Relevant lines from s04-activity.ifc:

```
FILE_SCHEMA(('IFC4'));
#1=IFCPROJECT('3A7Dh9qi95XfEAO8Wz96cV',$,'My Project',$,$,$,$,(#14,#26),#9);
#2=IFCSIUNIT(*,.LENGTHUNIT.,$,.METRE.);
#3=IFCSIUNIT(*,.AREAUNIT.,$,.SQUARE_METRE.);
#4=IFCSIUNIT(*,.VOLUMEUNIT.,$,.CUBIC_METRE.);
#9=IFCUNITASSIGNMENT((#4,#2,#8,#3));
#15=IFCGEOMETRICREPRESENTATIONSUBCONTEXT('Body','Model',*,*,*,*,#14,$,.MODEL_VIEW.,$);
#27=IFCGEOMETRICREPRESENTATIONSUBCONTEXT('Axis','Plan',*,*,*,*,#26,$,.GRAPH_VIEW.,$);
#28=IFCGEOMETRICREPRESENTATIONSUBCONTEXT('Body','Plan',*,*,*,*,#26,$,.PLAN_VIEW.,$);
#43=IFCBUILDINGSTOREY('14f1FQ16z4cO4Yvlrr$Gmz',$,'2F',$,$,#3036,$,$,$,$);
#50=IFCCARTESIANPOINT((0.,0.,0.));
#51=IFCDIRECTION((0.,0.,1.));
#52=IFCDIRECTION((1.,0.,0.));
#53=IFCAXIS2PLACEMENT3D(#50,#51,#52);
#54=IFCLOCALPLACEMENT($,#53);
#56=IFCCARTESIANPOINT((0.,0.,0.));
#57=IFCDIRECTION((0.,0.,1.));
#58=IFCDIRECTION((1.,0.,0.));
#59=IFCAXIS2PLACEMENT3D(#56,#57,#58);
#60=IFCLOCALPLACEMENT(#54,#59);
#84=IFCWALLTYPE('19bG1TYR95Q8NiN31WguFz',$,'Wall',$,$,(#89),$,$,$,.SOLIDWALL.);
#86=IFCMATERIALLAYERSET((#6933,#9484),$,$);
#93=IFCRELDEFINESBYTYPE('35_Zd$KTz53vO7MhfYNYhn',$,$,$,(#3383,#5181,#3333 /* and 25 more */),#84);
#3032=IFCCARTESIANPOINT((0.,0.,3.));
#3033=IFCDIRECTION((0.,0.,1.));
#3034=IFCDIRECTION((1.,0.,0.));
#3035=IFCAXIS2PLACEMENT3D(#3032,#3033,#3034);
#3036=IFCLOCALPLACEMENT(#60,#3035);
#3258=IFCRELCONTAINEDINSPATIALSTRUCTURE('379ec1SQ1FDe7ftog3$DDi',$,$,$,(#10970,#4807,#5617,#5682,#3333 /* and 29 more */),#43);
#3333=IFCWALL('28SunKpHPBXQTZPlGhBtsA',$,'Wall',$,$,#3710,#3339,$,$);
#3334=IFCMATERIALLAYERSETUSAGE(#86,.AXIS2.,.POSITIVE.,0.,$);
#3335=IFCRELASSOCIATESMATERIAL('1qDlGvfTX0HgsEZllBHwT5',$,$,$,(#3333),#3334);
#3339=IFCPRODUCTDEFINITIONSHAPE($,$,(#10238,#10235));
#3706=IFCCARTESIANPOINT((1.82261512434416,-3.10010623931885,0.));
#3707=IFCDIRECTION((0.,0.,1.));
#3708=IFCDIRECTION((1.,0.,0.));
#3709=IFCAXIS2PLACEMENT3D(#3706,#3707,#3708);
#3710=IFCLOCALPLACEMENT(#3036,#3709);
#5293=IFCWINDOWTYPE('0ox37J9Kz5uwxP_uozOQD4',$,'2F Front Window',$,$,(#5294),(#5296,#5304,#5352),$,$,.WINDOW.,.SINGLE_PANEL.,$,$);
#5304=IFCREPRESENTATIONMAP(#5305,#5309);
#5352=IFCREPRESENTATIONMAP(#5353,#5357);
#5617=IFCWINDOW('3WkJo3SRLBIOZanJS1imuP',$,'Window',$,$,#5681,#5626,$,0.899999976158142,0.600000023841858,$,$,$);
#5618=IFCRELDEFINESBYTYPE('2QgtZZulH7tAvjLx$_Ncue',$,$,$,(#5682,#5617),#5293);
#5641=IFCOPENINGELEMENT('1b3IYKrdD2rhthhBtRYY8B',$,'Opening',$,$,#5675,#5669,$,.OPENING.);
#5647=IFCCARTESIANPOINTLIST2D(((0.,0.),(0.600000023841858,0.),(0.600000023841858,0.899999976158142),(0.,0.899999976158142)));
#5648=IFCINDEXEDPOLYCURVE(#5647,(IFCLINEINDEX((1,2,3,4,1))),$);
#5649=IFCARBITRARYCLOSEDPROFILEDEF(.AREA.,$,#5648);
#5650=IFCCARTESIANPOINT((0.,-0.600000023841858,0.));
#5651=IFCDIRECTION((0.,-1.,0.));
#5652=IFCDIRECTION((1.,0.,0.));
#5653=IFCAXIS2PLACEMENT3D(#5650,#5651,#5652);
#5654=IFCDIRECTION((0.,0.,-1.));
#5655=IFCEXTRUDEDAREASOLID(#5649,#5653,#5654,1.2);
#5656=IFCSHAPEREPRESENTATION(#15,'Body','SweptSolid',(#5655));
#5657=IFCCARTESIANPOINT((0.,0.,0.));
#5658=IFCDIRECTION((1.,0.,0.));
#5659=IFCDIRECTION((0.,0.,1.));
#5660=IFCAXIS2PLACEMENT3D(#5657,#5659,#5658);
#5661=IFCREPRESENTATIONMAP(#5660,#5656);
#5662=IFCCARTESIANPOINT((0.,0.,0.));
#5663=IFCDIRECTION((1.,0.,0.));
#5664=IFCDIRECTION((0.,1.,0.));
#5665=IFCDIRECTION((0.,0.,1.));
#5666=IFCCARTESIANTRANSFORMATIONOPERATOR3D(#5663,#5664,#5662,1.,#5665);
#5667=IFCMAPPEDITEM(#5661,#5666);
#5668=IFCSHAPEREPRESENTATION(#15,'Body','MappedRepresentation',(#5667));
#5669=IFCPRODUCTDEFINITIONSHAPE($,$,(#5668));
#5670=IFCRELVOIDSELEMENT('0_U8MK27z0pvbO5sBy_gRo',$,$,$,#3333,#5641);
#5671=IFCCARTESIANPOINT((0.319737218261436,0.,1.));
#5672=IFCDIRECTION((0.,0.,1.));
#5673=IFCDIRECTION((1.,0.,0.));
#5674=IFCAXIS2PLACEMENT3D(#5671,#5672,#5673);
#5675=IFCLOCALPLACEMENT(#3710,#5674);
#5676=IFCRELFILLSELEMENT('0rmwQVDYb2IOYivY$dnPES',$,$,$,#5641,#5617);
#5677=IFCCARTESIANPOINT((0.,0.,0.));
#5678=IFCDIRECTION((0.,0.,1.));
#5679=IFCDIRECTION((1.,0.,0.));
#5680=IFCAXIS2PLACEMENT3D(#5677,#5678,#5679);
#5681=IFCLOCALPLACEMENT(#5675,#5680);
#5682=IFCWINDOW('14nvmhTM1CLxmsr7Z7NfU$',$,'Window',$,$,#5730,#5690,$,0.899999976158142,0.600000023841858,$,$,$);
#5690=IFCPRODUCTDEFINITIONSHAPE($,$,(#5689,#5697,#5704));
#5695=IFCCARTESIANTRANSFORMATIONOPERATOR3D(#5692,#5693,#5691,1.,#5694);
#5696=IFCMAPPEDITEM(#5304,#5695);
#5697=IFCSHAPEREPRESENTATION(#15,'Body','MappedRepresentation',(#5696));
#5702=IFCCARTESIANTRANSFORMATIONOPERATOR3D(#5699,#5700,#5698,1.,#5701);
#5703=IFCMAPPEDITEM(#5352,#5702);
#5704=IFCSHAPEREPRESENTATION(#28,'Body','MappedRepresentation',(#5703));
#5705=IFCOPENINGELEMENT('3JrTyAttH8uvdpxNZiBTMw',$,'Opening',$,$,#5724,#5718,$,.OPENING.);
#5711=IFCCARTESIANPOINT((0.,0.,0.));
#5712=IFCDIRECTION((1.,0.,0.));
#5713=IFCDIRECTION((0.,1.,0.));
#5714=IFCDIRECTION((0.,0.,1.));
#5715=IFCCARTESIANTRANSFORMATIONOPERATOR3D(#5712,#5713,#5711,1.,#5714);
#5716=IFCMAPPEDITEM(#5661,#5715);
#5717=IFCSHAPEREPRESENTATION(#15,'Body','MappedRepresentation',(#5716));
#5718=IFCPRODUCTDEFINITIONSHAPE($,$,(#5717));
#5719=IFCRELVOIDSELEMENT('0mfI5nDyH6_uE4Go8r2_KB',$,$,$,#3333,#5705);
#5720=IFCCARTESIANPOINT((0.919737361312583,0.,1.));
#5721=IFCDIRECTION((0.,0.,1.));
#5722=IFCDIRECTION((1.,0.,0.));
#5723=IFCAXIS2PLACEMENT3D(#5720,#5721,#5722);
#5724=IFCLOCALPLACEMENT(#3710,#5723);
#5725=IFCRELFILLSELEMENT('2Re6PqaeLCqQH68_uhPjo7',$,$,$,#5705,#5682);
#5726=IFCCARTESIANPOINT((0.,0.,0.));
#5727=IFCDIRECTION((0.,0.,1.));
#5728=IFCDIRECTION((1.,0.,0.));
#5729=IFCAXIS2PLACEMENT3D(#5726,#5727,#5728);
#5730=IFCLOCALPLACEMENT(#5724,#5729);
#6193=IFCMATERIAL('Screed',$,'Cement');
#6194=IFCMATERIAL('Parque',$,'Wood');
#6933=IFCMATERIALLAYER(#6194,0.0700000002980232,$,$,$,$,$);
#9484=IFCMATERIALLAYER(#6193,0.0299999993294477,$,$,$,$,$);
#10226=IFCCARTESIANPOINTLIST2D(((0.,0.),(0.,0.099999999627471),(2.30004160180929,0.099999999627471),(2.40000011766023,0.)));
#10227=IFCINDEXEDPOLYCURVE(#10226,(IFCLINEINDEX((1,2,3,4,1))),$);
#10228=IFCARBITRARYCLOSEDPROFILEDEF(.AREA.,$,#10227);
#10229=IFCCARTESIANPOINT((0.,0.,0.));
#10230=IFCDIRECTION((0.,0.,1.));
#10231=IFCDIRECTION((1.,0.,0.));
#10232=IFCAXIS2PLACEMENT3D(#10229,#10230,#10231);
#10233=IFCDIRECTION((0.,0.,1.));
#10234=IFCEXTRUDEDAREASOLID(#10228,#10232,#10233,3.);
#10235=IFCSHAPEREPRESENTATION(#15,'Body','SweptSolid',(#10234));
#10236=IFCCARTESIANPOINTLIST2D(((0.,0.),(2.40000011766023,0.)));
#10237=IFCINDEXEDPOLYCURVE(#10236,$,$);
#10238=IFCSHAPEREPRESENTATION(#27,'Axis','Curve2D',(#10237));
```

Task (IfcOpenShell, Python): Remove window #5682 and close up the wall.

```python
import ifcopenshell
import ifcopenshell.api.feature
import ifcopenshell.api.root
import ifcopenshell.geom
import ifcopenshell.util.shape

model = ifcopenshell.open("s04-activity.ifc")
settings = ifcopenshell.geom.settings()


def volume(element):
    """Net volume in cubic metres, openings subtracted."""
    shape = ifcopenshell.geom.create_shape(settings, element)
    return ifcopenshell.util.shape.get_volume(shape.geometry)


window = model.by_id(5682)
opening = window.FillsVoids[0].RelatingOpeningElement
wall = opening.VoidsElements[0].RelatingBuildingElement
before = volume(wall)

ifcopenshell.api.root.remove_product(model, product=window)
ifcopenshell.api.feature.remove_feature(model, feature=opening)

after = volume(wall)

print(f"wall volume {before:.3f} -> {after:.3f} m3")

model.write("s04-activity_updated.ifc")
```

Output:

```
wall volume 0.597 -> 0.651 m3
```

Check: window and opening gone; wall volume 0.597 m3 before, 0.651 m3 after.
